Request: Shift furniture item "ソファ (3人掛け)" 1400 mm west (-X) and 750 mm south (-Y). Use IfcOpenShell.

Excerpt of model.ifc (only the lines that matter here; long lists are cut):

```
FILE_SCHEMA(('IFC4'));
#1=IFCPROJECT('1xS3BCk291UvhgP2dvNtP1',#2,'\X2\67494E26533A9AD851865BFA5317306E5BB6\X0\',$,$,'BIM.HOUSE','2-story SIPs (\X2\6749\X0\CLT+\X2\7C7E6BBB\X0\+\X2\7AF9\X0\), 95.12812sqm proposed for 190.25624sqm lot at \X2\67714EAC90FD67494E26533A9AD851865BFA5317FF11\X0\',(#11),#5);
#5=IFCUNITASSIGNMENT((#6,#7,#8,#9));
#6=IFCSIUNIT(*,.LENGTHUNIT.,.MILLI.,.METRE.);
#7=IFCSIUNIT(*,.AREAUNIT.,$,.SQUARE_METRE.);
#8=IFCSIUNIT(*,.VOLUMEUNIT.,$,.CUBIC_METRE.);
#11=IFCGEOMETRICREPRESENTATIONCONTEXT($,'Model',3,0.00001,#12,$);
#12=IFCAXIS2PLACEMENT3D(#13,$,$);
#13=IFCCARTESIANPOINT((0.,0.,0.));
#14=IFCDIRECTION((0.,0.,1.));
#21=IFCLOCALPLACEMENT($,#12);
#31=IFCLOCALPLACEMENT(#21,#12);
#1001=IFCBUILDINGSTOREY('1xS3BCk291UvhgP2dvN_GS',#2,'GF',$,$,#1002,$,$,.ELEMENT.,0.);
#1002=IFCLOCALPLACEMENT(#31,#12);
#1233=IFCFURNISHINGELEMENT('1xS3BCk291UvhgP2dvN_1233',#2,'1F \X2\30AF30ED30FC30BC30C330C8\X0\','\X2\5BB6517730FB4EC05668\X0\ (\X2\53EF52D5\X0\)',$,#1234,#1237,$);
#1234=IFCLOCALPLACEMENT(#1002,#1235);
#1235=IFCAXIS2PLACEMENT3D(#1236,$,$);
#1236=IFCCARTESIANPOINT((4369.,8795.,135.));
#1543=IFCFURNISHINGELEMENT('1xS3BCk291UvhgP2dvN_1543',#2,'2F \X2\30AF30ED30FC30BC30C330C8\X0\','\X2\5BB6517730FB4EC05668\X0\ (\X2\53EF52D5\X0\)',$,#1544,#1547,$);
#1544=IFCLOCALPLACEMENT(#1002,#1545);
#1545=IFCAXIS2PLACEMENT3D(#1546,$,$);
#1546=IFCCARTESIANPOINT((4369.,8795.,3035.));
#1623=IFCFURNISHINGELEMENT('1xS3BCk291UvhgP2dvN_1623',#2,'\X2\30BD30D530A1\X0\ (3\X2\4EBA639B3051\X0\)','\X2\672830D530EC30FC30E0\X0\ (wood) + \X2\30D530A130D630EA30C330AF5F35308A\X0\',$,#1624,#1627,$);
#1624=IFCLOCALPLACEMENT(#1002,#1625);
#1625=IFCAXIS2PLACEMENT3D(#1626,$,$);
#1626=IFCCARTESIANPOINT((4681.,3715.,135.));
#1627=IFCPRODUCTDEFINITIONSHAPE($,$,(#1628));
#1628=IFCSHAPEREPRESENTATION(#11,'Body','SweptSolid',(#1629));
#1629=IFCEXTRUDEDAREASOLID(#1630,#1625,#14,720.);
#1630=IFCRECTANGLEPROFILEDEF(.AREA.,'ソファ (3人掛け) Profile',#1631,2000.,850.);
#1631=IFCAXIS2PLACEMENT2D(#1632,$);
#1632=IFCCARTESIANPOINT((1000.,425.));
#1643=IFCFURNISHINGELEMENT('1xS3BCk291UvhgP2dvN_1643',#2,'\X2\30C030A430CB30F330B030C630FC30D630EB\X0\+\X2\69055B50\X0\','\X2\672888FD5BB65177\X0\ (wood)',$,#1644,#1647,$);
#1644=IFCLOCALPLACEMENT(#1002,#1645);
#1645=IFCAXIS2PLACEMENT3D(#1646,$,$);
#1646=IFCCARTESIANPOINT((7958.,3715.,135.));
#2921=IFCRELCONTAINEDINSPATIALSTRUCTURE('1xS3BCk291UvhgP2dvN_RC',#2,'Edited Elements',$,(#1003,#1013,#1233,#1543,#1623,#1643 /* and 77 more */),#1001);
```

```python
import ifcopenshell
import ifcopenshell.api.geometry
import ifcopenshell.util.placement
import ifcopenshell.util.unit

model = ifcopenshell.open("model.ifc")
unit_scale = ifcopenshell.util.unit.calculate_unit_scale(model)

item = model.by_guid("1xS3BCk291UvhgP2dvN_1623")
matrix = ifcopenshell.util.placement.get_local_placement(item.ObjectPlacement)
matrix[0, 3] -= 1.4 / unit_scale
matrix[1, 3] -= 0.75 / unit_scale
ifcopenshell.api.geometry.edit_object_placement(model, product=item, matrix=matrix, is_si=False)

print(ifcopenshell.util.placement.get_local_placement(item.ObjectPlacement).round(3) + 0.0)

model.write("model_rev.ifc")
```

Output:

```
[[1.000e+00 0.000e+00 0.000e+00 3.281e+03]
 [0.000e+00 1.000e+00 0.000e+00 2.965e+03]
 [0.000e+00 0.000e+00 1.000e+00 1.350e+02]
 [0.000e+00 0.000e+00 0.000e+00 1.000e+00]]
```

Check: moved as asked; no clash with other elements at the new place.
